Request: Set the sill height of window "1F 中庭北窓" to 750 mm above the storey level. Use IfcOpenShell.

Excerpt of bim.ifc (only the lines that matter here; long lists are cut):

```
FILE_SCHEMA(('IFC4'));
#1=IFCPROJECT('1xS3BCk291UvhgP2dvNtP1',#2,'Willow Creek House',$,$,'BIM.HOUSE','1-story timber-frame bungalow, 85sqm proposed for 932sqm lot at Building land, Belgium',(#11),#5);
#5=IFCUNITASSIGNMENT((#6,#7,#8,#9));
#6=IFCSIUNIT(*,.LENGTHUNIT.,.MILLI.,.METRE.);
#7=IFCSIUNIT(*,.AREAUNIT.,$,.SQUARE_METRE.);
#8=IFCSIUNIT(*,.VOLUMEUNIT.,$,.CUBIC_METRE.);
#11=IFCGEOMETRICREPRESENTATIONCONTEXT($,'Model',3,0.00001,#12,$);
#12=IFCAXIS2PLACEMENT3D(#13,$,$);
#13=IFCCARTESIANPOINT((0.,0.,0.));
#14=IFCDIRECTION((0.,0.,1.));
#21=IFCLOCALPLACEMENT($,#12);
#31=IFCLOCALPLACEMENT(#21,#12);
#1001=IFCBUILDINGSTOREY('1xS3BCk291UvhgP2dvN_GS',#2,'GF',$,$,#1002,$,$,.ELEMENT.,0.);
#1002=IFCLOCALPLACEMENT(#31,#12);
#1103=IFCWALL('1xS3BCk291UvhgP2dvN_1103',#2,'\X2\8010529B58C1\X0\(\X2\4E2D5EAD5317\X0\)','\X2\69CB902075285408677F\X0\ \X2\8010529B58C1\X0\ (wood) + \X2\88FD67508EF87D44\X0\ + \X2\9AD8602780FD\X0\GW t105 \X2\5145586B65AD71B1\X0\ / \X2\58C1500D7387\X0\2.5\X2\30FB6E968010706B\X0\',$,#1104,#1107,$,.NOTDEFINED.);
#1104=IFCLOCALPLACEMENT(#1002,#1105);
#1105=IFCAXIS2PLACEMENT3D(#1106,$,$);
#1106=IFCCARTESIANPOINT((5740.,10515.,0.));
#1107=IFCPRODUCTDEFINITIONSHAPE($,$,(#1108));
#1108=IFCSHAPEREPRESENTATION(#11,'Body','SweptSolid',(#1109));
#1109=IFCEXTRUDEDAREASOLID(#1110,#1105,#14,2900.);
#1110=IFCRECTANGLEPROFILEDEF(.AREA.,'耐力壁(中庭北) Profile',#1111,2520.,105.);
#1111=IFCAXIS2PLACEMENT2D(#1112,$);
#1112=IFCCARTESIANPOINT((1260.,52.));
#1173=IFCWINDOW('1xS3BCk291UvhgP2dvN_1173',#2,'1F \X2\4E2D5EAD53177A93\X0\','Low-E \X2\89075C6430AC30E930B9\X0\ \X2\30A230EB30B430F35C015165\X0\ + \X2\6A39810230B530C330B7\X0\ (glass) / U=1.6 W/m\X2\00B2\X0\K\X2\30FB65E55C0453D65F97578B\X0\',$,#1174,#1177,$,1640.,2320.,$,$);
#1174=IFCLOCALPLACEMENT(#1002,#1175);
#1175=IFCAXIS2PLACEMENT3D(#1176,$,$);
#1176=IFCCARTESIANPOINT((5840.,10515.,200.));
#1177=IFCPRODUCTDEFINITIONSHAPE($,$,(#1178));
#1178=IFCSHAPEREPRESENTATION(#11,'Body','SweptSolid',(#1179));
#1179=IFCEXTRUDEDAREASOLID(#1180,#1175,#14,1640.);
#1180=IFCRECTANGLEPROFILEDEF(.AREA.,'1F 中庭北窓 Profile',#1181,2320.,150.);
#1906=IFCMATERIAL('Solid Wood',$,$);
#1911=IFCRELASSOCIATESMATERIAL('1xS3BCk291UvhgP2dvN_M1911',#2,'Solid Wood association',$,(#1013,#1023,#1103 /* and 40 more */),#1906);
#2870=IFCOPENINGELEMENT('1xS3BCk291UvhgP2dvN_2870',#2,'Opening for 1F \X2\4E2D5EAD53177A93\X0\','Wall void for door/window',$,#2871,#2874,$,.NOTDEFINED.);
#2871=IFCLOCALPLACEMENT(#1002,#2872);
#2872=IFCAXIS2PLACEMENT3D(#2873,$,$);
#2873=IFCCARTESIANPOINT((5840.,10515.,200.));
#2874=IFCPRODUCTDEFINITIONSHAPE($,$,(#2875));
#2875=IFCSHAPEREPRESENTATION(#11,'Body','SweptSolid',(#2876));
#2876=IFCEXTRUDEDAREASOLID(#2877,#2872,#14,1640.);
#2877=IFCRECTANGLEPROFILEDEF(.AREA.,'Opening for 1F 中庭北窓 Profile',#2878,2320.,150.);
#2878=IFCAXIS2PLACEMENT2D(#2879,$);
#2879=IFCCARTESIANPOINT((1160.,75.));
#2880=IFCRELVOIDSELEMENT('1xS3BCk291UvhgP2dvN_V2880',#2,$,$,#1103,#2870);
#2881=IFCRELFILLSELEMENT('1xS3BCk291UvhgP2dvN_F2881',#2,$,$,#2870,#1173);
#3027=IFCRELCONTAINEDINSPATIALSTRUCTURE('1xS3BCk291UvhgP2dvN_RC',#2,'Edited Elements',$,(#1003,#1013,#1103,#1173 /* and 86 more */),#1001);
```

```python
import numpy as np
import ifcopenshell
import ifcopenshell.api.geometry
import ifcopenshell.geom
import ifcopenshell.util.element
import ifcopenshell.util.placement
import ifcopenshell.util.shape
import ifcopenshell.util.unit

model = ifcopenshell.open("bim.ifc")
unit_scale = ifcopenshell.util.unit.calculate_unit_scale(model)

window = model.by_guid("1xS3BCk291UvhgP2dvN_1173")
opening = window.FillsVoids[0].RelatingOpeningElement
storey = ifcopenshell.util.element.get_container(window, ifc_class="IfcBuildingStorey")
level = ifcopenshell.util.placement.get_local_placement(storey.ObjectPlacement)[2, 3]

# The opening's origin need not be at the sill, so measure its lowest point.
shape = ifcopenshell.geom.create_shape(ifcopenshell.geom.settings(), opening)
bottom = ifcopenshell.util.shape.get_shape_bottom_elevation(shape, shape.geometry) / unit_scale
dz = level + 0.75 / unit_scale - bottom

shift = np.array([0.0, 0.0, dz])
# The window is not placed relative to its opening, so move both.
for product in (opening, window):
    matrix = ifcopenshell.util.placement.get_local_placement(product.ObjectPlacement)
    matrix[:3, 3] += shift
    ifcopenshell.api.geometry.edit_object_placement(model, product=product, matrix=matrix, is_si=False)

print(f"moved by {dz * unit_scale:+.3f} m")

model.write("bim-out.ifc")
```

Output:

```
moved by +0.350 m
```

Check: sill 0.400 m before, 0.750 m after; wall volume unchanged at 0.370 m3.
